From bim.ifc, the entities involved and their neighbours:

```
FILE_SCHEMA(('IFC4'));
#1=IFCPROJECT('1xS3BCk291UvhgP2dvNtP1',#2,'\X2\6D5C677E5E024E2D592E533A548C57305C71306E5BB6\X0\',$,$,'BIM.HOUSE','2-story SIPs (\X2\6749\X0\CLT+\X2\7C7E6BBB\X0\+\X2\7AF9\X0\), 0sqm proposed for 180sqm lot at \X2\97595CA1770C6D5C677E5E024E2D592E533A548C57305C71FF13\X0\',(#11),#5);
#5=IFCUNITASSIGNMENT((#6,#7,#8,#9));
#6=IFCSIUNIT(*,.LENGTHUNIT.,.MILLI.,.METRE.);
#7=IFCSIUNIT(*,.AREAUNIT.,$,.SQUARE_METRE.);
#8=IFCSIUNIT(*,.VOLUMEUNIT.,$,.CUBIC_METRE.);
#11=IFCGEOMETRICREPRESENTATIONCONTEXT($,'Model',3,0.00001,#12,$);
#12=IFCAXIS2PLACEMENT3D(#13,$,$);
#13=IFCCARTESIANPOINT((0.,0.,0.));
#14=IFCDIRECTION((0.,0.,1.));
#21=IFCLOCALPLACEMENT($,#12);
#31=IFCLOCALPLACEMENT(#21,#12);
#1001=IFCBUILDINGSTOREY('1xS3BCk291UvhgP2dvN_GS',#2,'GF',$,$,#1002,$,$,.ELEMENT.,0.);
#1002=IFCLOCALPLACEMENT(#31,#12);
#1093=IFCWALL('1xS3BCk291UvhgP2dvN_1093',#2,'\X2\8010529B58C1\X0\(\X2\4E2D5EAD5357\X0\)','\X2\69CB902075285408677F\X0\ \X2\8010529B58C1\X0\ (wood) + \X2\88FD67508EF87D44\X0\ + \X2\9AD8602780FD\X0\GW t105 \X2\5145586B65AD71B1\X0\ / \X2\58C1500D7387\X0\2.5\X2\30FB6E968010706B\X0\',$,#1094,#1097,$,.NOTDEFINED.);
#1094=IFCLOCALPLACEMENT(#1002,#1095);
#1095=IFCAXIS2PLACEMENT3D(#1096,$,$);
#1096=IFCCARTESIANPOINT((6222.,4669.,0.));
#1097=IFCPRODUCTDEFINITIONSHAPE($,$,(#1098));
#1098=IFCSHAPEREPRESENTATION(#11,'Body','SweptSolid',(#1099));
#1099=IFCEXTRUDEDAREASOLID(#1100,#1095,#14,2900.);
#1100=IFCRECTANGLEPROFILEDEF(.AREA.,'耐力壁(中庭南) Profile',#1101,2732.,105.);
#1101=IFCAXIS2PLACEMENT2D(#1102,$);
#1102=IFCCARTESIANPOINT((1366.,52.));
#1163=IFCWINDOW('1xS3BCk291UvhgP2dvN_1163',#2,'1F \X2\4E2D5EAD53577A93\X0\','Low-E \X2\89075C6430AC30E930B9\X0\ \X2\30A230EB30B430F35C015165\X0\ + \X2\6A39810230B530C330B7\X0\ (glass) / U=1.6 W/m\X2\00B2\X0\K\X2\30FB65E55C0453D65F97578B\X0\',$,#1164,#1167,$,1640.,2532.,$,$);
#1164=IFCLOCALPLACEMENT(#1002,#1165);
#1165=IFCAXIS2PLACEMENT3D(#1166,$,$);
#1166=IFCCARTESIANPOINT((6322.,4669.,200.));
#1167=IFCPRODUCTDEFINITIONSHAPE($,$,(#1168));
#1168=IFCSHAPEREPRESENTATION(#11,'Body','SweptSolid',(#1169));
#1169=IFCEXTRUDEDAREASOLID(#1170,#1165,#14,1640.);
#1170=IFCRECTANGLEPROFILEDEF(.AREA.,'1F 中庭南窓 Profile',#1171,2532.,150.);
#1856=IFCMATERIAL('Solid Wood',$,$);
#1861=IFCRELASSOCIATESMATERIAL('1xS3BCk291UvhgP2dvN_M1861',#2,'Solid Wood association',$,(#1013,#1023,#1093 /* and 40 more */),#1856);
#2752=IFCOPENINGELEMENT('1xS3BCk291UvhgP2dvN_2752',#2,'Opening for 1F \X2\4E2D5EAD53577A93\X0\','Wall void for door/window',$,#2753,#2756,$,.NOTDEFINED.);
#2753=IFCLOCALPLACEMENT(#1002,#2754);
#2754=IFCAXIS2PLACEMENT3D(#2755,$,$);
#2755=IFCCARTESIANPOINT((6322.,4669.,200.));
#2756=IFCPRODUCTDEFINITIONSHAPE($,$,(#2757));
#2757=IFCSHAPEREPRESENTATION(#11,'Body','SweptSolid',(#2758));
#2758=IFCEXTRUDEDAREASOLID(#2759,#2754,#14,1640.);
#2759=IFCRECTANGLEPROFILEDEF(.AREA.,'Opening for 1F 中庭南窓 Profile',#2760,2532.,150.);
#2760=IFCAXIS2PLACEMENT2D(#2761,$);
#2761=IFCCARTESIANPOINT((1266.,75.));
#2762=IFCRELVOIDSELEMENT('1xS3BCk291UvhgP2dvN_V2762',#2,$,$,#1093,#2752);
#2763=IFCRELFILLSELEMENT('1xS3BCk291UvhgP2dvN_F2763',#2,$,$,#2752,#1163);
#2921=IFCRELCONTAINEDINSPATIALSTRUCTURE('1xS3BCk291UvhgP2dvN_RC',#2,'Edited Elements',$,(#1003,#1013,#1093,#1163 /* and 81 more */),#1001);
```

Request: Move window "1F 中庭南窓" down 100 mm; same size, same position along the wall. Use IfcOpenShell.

```python
import numpy as np
import ifcopenshell
import ifcopenshell.api.geometry
import ifcopenshell.util.placement
import ifcopenshell.util.unit

model = ifcopenshell.open("bim.ifc")
unit_scale = ifcopenshell.util.unit.calculate_unit_scale(model)

window = model.by_guid("1xS3BCk291UvhgP2dvN_1163")
opening = window.FillsVoids[0].RelatingOpeningElement
dz = -0.1 / unit_scale

shift = np.array([0.0, 0.0, dz])
# The window is not placed relative to its opening, so move both.
for product in (opening, window):
    matrix = ifcopenshell.util.placement.get_local_placement(product.ObjectPlacement)
    matrix[:3, 3] += shift
    ifcopenshell.api.geometry.edit_object_placement(model, product=product, matrix=matrix, is_si=False)

print(f"moved by {dz * unit_scale:+.3f} m")

model.write("bim_v2.ifc")
```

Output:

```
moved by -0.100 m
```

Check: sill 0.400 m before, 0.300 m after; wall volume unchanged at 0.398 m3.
